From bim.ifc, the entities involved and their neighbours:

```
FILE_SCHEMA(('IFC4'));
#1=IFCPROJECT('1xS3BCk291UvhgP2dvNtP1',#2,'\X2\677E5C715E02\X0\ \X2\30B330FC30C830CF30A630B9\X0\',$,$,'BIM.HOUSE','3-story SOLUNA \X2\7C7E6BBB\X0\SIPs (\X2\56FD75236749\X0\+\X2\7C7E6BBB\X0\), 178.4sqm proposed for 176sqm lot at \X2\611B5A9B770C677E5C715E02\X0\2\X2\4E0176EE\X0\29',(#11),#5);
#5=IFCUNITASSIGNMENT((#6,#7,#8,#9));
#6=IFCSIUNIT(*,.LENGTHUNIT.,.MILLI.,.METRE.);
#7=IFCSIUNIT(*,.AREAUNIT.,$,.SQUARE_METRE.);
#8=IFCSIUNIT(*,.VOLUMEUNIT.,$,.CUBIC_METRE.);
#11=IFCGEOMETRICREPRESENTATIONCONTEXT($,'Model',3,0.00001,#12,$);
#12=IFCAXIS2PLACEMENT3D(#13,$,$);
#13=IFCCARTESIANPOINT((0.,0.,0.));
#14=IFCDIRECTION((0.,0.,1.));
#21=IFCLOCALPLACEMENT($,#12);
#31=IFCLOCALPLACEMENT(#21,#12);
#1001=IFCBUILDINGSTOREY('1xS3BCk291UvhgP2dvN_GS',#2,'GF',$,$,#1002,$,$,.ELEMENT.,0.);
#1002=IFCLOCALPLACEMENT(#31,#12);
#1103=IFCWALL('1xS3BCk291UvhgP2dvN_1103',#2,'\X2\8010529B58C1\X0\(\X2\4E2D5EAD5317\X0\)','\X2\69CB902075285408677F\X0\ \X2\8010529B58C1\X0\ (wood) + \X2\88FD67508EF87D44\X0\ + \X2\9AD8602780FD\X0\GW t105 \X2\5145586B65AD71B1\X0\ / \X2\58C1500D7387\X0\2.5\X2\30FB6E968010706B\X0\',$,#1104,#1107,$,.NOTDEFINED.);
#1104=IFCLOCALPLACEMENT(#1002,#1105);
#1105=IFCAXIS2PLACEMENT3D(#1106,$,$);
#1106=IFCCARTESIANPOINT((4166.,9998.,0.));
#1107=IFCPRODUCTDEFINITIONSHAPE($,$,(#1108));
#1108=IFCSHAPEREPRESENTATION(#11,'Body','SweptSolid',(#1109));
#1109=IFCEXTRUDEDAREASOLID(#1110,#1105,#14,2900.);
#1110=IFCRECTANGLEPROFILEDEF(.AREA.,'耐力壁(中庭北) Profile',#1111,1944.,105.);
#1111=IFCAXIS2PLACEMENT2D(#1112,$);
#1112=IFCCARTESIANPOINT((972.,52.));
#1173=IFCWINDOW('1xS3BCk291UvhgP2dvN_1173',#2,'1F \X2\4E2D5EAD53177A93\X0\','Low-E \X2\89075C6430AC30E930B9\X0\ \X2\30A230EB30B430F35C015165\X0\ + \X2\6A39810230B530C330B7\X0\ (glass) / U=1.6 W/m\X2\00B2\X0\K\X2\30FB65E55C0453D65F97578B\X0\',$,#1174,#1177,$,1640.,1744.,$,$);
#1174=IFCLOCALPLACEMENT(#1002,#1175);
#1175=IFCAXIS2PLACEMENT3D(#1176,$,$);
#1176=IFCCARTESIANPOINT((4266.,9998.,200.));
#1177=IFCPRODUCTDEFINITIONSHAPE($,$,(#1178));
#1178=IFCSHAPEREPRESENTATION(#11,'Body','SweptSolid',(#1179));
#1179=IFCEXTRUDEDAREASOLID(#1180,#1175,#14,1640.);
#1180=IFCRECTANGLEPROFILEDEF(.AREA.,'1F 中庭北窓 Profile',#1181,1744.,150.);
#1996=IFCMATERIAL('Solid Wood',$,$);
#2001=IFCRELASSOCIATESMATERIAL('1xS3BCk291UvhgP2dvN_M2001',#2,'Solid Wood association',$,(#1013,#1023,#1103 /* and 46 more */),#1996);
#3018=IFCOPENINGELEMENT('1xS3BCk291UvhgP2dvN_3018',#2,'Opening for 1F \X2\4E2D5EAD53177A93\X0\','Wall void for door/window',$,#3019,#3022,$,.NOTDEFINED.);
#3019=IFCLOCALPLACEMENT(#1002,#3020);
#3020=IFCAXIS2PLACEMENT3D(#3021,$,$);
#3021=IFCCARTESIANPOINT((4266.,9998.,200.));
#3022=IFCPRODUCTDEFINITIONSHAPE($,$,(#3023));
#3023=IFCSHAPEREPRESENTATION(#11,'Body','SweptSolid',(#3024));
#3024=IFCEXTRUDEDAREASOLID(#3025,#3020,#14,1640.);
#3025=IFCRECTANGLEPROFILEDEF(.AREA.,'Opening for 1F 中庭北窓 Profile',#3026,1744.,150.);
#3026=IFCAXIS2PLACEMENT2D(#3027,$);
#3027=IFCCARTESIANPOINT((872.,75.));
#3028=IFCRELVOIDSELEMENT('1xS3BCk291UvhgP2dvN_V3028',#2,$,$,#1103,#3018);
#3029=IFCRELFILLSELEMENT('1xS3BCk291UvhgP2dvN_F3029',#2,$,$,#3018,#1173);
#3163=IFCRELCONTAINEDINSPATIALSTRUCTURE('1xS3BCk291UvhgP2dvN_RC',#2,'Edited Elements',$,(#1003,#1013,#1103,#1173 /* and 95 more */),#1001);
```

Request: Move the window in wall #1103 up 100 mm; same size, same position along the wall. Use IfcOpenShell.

```python
import numpy as np
import ifcopenshell
import ifcopenshell.api.geometry
import ifcopenshell.util.placement
import ifcopenshell.util.unit

model = ifcopenshell.open("bim.ifc")
unit_scale = ifcopenshell.util.unit.calculate_unit_scale(model)

window = model.by_guid("1xS3BCk291UvhgP2dvN_1173")
opening = window.FillsVoids[0].RelatingOpeningElement
dz = 100.0

shift = np.array([0.0, 0.0, dz])
# The window is not placed relative to its opening, so move both.
for product in (opening, window):
    matrix = ifcopenshell.util.placement.get_local_placement(product.ObjectPlacement)
    matrix[:3, 3] += shift
    ifcopenshell.api.geometry.edit_object_placement(model, product=product, matrix=matrix, is_si=False)

print(f"moved by {dz * unit_scale:+.3f} m")

model.write("bim_edited.ifc")
```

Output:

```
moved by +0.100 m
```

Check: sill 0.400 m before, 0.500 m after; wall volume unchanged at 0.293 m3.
